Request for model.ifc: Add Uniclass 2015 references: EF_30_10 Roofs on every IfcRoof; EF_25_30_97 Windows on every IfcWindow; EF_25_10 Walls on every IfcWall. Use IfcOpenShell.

First a look at what the model holds.

```python
import ifcopenshell

model = ifcopenshell.open("model.ifc")
print(model.schema)
print("classifications:", [c.Name for c in model.by_type("IfcClassification")])
for ifc_class in ("IfcDoor", "IfcRoof", "IfcStair", "IfcWall", "IfcWindow"):
    print(ifc_class, len(model.by_type(ifc_class)))
```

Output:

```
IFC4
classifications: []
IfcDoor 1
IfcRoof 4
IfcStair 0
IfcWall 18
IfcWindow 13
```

```python
import ifcopenshell
import ifcopenshell.api.classification

model = ifcopenshell.open("model.ifc")

system = ifcopenshell.api.classification.add_classification(model, classification="Uniclass 2015")

codes = {
    "IfcRoof": ("EF_30_10", "Roofs"),
    "IfcWindow": ("EF_25_30_97", "Windows"),
    "IfcWall": ("EF_25_10", "Walls"),
}
for ifc_class, (code, name) in codes.items():
    products = model.by_type(ifc_class)
    ifcopenshell.api.classification.add_reference(
        model, products=products, classification=system, identification=code, name=name
    )
    print(code, len(products))

model.write("model-out.ifc")
```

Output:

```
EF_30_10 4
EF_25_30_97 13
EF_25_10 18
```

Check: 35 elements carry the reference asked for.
